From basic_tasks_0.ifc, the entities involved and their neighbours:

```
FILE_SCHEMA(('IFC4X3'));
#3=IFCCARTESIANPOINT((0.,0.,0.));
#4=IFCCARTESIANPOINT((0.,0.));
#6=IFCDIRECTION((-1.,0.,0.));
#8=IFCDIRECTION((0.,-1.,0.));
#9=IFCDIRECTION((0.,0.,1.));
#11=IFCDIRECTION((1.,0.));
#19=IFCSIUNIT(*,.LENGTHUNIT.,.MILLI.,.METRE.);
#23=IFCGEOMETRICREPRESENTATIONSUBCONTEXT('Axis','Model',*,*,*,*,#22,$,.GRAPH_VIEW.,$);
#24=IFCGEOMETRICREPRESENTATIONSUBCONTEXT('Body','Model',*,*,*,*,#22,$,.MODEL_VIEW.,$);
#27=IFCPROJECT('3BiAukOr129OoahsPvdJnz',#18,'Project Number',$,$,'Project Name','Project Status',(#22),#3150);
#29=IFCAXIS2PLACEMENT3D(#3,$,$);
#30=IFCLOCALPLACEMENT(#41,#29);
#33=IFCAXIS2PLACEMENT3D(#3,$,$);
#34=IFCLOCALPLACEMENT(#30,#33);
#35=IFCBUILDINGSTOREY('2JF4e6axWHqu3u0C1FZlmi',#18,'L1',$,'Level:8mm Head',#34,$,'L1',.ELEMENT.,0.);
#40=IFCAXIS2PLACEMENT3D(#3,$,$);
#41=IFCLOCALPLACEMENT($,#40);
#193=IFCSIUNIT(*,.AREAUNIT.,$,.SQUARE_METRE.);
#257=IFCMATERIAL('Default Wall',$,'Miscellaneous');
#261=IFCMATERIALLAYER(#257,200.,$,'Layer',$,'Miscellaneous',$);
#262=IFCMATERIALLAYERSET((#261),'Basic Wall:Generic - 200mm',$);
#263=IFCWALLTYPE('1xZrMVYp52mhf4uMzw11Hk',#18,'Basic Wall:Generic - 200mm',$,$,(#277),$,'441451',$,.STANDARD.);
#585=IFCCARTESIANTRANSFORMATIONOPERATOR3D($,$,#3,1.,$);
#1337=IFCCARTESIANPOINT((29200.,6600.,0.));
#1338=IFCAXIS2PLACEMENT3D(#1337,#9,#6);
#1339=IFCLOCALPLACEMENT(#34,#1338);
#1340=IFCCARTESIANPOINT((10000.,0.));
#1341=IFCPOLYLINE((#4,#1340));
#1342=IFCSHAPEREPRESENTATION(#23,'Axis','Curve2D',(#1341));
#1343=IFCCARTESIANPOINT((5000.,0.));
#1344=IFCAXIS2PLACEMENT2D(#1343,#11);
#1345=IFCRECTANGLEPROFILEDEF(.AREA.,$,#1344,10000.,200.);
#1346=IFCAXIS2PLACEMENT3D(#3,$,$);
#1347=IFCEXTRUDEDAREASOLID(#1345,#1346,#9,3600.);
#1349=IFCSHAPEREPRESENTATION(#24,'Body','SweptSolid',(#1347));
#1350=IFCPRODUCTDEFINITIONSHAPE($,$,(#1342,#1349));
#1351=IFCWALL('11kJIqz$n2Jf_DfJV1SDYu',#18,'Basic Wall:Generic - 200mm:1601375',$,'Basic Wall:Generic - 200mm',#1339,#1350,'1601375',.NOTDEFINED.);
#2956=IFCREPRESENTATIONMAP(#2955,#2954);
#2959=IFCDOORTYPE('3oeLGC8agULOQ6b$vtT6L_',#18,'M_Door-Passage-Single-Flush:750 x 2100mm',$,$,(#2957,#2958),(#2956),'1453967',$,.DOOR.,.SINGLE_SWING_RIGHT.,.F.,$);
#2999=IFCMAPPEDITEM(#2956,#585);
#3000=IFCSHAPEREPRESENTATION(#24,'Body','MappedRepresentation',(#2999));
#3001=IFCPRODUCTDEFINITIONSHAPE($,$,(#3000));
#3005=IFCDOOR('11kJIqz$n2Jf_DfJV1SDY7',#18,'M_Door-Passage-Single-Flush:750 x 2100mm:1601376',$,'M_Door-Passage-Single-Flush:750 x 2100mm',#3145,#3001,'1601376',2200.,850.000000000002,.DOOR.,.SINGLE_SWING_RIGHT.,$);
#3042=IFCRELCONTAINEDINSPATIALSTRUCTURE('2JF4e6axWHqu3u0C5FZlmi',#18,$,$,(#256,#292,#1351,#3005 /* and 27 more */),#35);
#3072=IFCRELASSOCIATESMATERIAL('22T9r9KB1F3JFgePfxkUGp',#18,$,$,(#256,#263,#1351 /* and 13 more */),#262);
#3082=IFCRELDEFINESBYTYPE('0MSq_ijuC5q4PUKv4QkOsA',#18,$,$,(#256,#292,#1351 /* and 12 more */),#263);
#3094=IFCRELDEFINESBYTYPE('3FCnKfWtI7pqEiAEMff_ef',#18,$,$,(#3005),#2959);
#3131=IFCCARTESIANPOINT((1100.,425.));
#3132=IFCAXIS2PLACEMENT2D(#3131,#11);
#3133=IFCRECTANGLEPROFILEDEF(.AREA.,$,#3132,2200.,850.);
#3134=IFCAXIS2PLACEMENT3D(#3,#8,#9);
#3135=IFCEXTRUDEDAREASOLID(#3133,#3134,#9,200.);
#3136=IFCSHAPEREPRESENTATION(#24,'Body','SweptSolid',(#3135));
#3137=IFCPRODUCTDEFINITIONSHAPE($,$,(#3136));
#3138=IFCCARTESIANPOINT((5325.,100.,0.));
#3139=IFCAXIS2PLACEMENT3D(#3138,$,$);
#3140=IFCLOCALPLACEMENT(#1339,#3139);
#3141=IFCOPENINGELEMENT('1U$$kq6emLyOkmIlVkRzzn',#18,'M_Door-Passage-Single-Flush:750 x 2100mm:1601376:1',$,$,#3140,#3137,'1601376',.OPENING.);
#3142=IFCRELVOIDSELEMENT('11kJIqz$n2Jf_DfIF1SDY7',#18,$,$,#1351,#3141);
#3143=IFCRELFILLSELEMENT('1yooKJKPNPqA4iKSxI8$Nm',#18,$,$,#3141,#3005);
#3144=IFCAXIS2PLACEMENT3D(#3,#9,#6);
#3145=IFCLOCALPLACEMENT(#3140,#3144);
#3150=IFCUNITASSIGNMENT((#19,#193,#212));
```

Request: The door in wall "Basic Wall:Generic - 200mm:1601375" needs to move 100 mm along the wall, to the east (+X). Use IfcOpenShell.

```python
import ifcopenshell
import ifcopenshell.api.geometry
import ifcopenshell.util.placement

model = ifcopenshell.open("basic_tasks_0.ifc")

door = model.by_id(3005)
opening = door.FillsVoids[0].RelatingOpeningElement
wall = opening.VoidsElements[0].RelatingBuildingElement

wall_matrix = ifcopenshell.util.placement.get_local_placement(wall.ObjectPlacement)
shift = wall_matrix[:3, 0] * -100.0
before = ifcopenshell.util.placement.get_local_placement(door.ObjectPlacement)[:3, 3].copy()

# The door is placed relative to its opening, so it follows when the opening moves.
matrix = ifcopenshell.util.placement.get_local_placement(opening.ObjectPlacement)
matrix[:3, 3] += shift
ifcopenshell.api.geometry.edit_object_placement(
    model, product=opening, matrix=matrix, is_si=False, should_transform_children=True
)

after = ifcopenshell.util.placement.get_local_placement(door.ObjectPlacement)[:3, 3]
print("door moved by", (after - before).round(3) + 0.0)

model.write("basic_tasks_0_rev.ifc")
```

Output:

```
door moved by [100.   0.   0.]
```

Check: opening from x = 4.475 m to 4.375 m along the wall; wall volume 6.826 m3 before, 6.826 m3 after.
